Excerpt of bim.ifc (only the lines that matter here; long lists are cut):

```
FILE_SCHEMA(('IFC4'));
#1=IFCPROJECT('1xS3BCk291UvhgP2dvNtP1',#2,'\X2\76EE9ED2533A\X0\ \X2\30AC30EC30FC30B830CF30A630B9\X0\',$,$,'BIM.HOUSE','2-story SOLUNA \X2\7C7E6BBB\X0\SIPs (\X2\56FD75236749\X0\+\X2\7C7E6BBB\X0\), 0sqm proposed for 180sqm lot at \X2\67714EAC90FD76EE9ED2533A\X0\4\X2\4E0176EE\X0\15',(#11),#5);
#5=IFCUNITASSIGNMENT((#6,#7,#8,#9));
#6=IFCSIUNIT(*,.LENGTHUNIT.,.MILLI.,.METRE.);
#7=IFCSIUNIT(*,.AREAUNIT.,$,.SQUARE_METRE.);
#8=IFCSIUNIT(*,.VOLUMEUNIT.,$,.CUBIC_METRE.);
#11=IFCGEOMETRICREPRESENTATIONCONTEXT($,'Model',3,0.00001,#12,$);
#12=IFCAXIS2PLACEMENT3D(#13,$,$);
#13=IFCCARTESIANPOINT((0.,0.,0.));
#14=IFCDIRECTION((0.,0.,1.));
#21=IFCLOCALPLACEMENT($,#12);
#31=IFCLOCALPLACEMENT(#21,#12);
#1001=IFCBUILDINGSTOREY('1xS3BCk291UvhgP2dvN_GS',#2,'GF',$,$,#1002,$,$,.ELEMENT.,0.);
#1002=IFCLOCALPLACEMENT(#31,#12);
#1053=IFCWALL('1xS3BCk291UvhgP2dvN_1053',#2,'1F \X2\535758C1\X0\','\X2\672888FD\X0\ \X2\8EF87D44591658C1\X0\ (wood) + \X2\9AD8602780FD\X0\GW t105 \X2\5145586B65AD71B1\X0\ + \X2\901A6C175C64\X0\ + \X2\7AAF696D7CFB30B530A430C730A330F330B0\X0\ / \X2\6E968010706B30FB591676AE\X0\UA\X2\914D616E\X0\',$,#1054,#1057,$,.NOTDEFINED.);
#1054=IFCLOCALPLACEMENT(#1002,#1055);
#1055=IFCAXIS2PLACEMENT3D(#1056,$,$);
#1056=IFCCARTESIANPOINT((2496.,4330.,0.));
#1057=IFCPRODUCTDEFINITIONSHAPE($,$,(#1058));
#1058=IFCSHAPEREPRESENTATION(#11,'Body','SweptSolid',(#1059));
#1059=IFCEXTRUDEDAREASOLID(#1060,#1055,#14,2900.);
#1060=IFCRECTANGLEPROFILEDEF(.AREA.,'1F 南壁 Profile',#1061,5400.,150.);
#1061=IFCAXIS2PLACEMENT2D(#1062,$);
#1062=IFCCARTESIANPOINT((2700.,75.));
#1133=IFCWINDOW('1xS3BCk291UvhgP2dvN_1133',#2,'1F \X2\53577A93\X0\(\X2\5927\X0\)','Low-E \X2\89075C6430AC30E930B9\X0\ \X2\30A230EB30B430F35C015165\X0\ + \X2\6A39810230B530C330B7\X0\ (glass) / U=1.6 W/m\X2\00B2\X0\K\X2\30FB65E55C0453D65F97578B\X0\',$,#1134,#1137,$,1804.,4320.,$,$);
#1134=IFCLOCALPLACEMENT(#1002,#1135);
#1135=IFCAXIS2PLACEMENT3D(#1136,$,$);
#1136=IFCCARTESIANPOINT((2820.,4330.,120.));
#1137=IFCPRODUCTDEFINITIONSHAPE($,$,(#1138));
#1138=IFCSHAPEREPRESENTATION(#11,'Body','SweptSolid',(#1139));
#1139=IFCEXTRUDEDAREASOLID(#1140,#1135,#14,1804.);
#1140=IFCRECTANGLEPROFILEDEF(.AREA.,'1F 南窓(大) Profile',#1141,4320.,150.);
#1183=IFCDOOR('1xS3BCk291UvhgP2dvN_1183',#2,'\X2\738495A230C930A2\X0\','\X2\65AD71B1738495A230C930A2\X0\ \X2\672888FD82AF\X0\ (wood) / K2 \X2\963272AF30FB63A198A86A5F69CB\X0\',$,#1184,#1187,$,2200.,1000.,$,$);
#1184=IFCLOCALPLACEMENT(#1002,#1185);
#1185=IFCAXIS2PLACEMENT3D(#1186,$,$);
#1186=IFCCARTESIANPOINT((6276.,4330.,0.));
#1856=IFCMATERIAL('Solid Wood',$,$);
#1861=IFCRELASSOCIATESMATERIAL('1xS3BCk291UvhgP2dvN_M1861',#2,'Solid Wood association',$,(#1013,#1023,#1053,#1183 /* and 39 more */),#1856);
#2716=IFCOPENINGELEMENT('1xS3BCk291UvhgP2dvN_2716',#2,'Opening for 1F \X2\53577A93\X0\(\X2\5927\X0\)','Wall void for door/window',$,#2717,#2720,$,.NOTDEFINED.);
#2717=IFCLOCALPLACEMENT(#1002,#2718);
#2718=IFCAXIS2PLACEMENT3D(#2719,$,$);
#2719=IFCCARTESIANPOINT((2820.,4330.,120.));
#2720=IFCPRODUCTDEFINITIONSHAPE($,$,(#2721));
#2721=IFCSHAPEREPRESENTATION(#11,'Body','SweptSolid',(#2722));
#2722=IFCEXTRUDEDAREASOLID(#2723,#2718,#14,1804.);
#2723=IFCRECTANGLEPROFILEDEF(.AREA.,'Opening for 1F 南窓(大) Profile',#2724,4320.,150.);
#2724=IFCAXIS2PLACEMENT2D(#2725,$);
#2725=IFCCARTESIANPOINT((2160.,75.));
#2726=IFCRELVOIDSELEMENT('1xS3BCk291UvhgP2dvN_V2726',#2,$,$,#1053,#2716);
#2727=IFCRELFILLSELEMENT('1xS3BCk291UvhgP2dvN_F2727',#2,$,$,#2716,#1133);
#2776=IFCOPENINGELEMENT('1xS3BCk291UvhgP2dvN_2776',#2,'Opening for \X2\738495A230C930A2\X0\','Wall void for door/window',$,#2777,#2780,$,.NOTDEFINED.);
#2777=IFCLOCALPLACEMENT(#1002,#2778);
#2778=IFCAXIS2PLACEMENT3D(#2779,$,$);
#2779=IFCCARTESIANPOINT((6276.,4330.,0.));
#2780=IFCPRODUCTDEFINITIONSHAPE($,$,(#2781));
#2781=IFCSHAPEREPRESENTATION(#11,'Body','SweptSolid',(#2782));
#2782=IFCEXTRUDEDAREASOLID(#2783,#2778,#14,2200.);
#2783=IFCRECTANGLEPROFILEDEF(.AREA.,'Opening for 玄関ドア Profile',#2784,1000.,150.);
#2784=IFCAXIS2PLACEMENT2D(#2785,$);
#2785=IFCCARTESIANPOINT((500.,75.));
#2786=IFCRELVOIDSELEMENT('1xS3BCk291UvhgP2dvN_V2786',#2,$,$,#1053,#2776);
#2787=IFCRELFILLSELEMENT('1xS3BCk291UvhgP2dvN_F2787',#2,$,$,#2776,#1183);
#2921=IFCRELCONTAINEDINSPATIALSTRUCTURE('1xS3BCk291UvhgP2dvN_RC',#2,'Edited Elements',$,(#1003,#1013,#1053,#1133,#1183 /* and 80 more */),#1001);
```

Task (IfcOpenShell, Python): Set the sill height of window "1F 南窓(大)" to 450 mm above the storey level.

```python
import numpy as np
import ifcopenshell
import ifcopenshell.api.geometry
import ifcopenshell.geom
import ifcopenshell.util.element
import ifcopenshell.util.placement
import ifcopenshell.util.shape
import ifcopenshell.util.unit

model = ifcopenshell.open("bim.ifc")
unit_scale = ifcopenshell.util.unit.calculate_unit_scale(model)

window = model.by_guid("1xS3BCk291UvhgP2dvN_1133")
opening = window.FillsVoids[0].RelatingOpeningElement
storey = ifcopenshell.util.element.get_container(window, ifc_class="IfcBuildingStorey")
level = ifcopenshell.util.placement.get_local_placement(storey.ObjectPlacement)[2, 3]

# The opening's origin need not be at the sill, so measure its lowest point.
shape = ifcopenshell.geom.create_shape(ifcopenshell.geom.settings(), opening)
bottom = ifcopenshell.util.shape.get_shape_bottom_elevation(shape, shape.geometry) / unit_scale
dz = level + 450.0 - bottom

shift = np.array([0.0, 0.0, dz])
# The window is not placed relative to its opening, so move both.
for product in (opening, window):
    matrix = ifcopenshell.util.placement.get_local_placement(product.ObjectPlacement)
    matrix[:3, 3] += shift
    ifcopenshell.api.geometry.edit_object_placement(model, product=product, matrix=matrix, is_si=False)

print(f"moved by {dz * unit_scale:+.3f} m")

model.write("bim-out.ifc")
```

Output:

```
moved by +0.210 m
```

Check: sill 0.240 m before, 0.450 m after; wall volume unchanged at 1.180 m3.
